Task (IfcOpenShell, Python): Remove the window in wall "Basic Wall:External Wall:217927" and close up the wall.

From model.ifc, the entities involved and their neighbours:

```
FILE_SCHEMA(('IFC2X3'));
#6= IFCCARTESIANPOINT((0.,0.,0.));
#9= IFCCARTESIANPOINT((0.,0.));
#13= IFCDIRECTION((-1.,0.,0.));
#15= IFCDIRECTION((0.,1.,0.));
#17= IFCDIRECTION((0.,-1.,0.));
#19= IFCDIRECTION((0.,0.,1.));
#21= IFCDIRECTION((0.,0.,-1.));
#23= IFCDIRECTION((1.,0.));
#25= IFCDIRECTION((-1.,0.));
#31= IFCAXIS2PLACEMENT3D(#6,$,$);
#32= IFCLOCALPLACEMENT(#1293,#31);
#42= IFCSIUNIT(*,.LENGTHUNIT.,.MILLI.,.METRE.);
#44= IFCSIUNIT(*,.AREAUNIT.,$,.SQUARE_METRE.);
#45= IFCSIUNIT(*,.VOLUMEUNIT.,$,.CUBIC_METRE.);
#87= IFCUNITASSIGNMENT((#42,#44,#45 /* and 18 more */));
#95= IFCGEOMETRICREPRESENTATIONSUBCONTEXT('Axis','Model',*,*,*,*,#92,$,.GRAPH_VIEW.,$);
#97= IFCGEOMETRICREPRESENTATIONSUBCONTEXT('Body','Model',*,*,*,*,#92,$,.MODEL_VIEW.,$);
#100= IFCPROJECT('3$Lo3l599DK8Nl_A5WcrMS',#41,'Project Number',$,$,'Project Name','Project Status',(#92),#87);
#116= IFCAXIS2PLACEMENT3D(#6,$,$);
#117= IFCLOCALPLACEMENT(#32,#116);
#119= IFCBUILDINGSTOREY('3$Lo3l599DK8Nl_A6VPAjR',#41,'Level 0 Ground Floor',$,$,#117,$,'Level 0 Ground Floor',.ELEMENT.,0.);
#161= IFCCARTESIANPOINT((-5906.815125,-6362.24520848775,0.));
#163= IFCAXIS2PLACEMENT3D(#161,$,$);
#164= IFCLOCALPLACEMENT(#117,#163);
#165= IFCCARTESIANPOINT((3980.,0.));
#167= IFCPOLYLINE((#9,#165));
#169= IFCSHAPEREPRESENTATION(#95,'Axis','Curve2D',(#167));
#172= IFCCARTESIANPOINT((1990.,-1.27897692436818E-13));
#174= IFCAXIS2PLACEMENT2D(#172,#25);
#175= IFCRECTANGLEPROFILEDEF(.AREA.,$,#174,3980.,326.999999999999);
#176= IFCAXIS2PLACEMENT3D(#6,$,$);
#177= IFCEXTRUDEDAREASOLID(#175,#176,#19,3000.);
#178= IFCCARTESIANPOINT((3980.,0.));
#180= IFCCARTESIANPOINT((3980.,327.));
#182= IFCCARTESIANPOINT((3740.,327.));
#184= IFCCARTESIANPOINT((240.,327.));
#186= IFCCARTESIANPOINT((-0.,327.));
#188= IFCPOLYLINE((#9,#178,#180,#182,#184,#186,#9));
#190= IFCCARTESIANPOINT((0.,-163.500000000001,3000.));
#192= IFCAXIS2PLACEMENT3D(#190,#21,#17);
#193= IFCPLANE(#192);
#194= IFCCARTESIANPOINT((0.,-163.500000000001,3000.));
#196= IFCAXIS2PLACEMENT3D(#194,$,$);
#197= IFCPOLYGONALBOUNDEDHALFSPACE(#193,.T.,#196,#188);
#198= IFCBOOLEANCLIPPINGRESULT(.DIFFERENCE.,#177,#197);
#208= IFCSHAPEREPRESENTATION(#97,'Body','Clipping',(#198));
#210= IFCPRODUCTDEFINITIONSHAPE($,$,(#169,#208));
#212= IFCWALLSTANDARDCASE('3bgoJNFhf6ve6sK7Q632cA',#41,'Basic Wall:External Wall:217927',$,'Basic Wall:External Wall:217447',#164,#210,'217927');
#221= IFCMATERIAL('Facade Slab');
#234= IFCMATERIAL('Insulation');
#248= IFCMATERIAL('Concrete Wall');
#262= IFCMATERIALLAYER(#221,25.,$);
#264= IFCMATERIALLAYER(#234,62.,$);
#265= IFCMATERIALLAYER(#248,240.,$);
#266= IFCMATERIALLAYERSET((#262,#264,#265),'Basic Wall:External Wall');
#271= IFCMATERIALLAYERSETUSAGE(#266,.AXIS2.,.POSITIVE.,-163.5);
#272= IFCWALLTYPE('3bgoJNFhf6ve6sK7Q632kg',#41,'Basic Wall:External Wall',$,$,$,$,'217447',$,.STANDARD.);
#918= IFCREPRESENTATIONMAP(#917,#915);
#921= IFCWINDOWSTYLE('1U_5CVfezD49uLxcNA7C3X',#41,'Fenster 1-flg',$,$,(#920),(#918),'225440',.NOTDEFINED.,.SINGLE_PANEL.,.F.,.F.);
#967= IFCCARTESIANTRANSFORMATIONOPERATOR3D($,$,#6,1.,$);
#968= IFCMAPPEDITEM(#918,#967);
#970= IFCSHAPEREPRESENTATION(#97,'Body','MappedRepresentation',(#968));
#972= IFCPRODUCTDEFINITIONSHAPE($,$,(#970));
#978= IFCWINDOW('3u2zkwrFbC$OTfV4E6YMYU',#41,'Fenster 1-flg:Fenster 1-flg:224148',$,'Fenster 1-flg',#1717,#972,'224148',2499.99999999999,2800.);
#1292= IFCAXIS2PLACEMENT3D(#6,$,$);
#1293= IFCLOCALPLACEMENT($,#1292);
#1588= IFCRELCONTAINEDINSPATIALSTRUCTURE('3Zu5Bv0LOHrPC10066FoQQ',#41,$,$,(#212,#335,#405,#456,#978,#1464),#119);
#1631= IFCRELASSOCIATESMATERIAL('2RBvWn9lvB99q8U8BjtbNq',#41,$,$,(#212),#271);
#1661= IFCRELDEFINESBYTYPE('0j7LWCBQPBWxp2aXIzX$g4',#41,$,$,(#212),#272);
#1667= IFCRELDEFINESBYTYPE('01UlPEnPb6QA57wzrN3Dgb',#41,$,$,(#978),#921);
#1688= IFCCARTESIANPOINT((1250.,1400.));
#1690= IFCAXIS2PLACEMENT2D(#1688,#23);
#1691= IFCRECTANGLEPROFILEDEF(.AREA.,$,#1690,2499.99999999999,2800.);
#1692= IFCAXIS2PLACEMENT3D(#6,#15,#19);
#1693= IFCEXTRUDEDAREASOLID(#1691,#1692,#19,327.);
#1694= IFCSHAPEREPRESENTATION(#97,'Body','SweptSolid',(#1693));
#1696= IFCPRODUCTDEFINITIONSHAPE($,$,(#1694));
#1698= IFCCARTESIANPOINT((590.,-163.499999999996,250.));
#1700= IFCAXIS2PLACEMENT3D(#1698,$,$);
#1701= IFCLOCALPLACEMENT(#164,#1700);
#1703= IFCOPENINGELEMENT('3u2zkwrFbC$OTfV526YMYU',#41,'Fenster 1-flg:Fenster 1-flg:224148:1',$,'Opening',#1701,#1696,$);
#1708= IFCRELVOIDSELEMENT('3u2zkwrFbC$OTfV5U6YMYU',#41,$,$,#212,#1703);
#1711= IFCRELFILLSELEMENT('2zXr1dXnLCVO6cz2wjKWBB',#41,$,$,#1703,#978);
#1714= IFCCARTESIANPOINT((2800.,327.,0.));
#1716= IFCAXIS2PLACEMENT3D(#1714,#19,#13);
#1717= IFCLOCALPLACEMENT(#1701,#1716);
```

```python
import ifcopenshell
import ifcopenshell.api.feature
import ifcopenshell.api.root
import ifcopenshell.geom
import ifcopenshell.util.shape

model = ifcopenshell.open("model.ifc")
settings = ifcopenshell.geom.settings()


def volume(element):
    """Net volume in cubic metres, openings subtracted."""
    shape = ifcopenshell.geom.create_shape(settings, element)
    return ifcopenshell.util.shape.get_volume(shape.geometry)


window = model.by_guid("3u2zkwrFbC$OTfV4E6YMYU")
opening = window.FillsVoids[0].RelatingOpeningElement
wall = opening.VoidsElements[0].RelatingBuildingElement
before = volume(wall)

ifcopenshell.api.root.remove_product(model, product=window)
ifcopenshell.api.feature.remove_feature(model, feature=opening)

after = volume(wall)

print(f"wall volume {before:.3f} -> {after:.3f} m3")

model.write("model_rev.ifc")
```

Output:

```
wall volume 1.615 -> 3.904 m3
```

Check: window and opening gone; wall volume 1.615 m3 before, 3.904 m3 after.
